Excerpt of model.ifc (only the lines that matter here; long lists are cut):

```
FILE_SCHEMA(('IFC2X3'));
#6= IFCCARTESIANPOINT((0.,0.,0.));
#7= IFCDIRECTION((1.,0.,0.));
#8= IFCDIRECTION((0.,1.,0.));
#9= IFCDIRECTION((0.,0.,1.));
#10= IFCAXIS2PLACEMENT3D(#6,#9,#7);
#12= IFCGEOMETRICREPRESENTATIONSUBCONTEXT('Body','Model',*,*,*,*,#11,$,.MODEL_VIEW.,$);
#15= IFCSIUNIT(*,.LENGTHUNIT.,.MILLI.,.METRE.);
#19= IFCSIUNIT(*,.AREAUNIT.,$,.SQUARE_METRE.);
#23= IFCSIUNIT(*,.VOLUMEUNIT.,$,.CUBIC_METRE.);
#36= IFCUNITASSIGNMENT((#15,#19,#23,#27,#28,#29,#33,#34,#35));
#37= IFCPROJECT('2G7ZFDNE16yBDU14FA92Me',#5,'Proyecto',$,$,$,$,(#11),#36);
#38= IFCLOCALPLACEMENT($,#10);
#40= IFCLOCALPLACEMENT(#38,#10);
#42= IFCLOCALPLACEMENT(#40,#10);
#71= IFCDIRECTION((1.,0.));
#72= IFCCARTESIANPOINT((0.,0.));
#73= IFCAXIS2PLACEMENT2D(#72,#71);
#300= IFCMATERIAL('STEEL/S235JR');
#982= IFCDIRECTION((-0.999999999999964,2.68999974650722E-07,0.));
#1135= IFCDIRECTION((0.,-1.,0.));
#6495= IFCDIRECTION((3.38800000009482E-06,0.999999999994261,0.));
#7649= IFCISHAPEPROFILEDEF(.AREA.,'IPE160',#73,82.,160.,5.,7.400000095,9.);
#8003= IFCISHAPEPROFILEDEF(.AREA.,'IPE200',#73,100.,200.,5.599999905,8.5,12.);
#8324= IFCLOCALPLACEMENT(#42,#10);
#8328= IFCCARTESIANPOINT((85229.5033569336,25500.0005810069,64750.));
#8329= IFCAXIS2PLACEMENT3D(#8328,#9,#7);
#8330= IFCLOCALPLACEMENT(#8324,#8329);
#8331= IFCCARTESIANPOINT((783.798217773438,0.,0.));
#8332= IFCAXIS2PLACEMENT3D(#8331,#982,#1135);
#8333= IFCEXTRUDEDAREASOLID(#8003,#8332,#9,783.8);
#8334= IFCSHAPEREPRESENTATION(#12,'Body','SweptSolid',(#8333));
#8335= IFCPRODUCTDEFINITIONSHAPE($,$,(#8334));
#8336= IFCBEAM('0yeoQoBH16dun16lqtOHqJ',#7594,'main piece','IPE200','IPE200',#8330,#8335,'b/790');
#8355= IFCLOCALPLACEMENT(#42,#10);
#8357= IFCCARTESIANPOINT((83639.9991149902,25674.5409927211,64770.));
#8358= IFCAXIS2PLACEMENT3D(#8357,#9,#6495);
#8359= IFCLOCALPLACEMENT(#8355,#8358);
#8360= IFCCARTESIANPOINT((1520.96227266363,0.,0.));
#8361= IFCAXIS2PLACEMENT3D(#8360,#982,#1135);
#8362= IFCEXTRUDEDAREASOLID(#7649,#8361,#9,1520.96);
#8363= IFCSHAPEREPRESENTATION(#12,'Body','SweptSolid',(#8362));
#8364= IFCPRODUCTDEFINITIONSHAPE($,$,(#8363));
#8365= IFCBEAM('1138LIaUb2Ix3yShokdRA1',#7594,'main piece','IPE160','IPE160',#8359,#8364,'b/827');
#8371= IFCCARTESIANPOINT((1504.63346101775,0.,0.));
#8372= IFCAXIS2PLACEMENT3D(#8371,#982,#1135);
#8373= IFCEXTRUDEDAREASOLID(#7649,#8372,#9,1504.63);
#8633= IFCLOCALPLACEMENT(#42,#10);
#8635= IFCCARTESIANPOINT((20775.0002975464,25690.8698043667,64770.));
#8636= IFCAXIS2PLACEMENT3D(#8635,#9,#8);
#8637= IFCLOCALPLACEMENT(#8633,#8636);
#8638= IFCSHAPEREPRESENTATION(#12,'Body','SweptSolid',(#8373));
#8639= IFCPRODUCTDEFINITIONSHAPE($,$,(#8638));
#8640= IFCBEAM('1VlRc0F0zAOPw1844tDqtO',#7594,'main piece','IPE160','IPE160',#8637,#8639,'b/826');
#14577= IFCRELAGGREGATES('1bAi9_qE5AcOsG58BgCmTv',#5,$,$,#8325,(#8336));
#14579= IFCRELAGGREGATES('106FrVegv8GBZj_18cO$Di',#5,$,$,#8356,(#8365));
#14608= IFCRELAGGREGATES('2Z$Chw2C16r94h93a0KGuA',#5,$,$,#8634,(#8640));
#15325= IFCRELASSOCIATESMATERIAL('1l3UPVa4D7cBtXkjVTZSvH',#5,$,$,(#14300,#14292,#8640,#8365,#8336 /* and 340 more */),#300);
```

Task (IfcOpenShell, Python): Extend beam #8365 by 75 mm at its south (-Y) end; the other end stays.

```python
import ifcopenshell
import ifcopenshell.util.representation

model = ifcopenshell.open("model.ifc")

member = model.by_guid("1138LIaUb2Ix3yShokdRA1")
change = 75.0

# The extrusion runs towards the end named, so only its depth changes.
body = ifcopenshell.util.representation.get_representation(member, "Model", "Body")
solid = body.Items[0]
old_length = solid.Depth
solid.Depth += change

print(f"length {old_length:g} -> {solid.Depth:g}")

model.write("model_v2.ifc")
```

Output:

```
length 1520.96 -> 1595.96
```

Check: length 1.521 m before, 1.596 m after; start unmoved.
